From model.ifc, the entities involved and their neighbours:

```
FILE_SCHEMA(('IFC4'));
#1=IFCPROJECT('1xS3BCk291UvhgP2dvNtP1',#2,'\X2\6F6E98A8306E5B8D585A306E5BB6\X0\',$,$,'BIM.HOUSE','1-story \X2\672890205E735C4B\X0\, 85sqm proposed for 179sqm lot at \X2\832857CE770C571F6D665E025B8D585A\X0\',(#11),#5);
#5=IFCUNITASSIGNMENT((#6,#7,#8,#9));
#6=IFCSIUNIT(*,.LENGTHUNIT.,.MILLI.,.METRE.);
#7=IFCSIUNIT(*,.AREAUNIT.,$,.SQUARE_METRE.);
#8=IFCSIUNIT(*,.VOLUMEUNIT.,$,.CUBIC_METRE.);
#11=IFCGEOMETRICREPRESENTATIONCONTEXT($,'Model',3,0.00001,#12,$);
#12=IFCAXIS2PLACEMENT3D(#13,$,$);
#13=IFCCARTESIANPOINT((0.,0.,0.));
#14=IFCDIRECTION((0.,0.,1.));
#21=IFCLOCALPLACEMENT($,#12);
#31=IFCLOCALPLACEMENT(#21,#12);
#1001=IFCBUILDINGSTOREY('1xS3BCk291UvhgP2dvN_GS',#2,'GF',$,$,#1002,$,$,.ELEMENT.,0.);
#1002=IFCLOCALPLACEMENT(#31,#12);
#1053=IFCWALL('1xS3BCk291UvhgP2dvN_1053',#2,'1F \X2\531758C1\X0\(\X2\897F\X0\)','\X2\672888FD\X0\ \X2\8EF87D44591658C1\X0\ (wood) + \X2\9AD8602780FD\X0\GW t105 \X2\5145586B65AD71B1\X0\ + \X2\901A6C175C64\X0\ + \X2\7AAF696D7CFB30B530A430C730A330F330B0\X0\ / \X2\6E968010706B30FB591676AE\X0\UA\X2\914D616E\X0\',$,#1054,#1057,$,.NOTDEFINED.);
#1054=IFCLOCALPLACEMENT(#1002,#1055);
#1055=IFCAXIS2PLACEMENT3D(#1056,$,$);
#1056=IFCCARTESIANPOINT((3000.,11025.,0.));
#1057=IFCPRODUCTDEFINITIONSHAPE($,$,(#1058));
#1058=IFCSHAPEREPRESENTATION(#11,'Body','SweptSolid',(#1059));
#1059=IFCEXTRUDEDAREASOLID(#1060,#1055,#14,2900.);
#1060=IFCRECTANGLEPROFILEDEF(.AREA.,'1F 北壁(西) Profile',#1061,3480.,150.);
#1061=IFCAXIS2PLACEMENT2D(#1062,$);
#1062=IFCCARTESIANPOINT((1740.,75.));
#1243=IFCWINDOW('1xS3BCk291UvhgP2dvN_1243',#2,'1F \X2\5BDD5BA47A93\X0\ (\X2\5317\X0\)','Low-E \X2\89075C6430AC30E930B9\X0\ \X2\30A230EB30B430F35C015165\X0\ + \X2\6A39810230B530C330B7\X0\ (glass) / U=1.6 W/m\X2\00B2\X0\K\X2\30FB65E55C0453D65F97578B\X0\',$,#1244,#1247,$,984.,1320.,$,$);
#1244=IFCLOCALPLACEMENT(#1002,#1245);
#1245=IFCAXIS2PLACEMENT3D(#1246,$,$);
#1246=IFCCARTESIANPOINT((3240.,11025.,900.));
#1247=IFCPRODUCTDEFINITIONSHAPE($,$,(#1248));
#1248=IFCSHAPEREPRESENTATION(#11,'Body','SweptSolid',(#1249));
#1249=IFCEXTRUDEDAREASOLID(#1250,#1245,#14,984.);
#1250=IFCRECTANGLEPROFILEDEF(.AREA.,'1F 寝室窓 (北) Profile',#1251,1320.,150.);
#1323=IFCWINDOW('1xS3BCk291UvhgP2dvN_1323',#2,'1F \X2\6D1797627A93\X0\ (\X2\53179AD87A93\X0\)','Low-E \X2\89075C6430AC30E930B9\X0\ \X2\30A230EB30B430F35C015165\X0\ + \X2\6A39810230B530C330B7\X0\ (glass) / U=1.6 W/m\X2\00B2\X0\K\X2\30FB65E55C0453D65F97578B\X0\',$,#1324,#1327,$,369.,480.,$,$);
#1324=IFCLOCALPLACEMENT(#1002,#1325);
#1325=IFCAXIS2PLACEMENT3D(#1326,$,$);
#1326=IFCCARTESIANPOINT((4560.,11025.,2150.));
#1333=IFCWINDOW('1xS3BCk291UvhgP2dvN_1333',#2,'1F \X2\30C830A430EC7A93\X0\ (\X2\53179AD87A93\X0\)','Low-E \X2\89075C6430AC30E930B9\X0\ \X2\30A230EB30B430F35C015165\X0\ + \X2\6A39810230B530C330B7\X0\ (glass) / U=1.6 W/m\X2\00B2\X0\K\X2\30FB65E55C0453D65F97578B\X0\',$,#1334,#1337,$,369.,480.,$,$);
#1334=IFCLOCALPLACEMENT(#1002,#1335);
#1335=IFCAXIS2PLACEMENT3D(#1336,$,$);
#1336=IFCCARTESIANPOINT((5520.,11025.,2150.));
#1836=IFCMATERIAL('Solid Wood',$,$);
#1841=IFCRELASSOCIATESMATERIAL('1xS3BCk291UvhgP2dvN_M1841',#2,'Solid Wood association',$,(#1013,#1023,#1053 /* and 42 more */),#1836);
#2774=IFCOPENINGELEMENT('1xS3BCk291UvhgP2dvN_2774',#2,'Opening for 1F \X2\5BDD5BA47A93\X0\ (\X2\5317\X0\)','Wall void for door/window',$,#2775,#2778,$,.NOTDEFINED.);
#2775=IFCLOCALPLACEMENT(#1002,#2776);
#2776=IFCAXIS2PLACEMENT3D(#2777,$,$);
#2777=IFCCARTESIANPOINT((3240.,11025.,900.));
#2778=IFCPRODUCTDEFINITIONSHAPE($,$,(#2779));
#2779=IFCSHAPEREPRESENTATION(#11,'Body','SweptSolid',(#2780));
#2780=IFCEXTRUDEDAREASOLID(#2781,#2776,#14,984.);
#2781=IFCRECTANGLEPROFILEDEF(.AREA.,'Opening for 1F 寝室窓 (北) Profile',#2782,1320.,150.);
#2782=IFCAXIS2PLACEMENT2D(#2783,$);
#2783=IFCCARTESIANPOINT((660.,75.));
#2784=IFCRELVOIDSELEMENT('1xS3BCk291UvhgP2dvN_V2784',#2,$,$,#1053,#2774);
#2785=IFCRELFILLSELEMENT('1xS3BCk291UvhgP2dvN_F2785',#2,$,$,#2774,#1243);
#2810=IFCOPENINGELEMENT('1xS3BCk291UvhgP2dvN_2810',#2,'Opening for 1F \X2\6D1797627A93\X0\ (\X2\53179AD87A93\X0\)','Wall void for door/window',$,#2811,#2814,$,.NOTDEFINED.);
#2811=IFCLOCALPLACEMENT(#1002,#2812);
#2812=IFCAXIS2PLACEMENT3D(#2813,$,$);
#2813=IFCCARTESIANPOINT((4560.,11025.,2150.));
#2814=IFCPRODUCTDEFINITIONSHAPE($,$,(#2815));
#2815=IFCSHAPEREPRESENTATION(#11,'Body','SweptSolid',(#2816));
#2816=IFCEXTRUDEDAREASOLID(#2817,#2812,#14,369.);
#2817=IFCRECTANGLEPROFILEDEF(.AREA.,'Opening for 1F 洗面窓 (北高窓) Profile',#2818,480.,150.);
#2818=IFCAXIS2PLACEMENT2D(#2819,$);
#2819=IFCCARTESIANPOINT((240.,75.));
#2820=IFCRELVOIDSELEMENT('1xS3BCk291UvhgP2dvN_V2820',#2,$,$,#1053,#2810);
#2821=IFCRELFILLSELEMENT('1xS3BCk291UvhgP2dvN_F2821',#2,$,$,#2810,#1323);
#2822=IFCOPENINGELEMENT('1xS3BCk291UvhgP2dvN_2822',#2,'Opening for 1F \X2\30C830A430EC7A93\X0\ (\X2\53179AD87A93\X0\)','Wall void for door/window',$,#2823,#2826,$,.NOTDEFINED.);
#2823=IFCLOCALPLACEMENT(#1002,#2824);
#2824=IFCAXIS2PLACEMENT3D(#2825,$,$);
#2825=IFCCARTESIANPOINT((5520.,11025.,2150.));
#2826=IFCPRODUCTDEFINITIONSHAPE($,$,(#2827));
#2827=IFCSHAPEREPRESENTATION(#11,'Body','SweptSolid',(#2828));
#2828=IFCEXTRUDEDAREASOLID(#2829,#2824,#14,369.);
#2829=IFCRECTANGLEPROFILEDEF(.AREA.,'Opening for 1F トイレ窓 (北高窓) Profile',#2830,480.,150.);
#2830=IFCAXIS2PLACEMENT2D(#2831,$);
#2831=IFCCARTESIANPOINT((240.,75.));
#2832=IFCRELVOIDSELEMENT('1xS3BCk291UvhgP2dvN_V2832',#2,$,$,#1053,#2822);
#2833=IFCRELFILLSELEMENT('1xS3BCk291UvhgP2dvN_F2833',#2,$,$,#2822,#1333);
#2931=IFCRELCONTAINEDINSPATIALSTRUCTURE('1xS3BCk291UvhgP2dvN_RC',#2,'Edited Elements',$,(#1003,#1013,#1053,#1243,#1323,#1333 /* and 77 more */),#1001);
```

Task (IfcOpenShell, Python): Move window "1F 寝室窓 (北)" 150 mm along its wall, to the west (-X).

```python
import ifcopenshell
import ifcopenshell.api.geometry
import ifcopenshell.util.placement

model = ifcopenshell.open("model.ifc")

window = model.by_id(1243)
opening = window.FillsVoids[0].RelatingOpeningElement
wall = opening.VoidsElements[0].RelatingBuildingElement

wall_matrix = ifcopenshell.util.placement.get_local_placement(wall.ObjectPlacement)
shift = wall_matrix[:3, 0] * -150.0
before = ifcopenshell.util.placement.get_local_placement(window.ObjectPlacement)[:3, 3].copy()

# The window is not placed relative to its opening, so move both.
for product in (opening, window):
    matrix = ifcopenshell.util.placement.get_local_placement(product.ObjectPlacement)
    matrix[:3, 3] += shift
    ifcopenshell.api.geometry.edit_object_placement(model, product=product, matrix=matrix, is_si=False)

after = ifcopenshell.util.placement.get_local_placement(window.ObjectPlacement)[:3, 3]
print("window moved by", (after - before).round(3) + 0.0)

model.write("model_edited.ifc")
```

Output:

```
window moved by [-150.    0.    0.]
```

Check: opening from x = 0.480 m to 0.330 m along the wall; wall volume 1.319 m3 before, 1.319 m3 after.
